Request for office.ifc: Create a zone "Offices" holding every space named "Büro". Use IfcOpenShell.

First a look at what the model holds.

```python
import ifcopenshell

model = ifcopenshell.open("office.ifc")
print(model.schema)
seen = {}
for space in model.by_type("IfcSpace"):
    seen[space.LongName] = seen.get(space.LongName, 0) + 1
for name, count in sorted(seen.items(), key=str):
    print(count, "x", name)
print("zones:", [z.Name for z in model.by_type("IfcZone")][:20])
```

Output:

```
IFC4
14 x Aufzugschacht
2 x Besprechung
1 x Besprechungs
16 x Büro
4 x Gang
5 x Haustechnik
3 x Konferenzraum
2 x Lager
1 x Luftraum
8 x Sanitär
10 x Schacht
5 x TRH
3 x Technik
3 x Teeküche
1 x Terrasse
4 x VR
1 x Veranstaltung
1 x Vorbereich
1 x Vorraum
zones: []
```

```python
import ifcopenshell
import ifcopenshell.api.group
import ifcopenshell.api.root

model = ifcopenshell.open("office.ifc")

names = {"Büro"}
spaces = [s for s in model.by_type("IfcSpace") if s.LongName in names]

zone = ifcopenshell.api.root.create_entity(model, ifc_class="IfcZone", name="Offices")
ifcopenshell.api.group.assign_group(model, products=spaces, group=zone)
print(len(spaces), "spaces in", zone.Name)

model.write("office-out.ifc")
```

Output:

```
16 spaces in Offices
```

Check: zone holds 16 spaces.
